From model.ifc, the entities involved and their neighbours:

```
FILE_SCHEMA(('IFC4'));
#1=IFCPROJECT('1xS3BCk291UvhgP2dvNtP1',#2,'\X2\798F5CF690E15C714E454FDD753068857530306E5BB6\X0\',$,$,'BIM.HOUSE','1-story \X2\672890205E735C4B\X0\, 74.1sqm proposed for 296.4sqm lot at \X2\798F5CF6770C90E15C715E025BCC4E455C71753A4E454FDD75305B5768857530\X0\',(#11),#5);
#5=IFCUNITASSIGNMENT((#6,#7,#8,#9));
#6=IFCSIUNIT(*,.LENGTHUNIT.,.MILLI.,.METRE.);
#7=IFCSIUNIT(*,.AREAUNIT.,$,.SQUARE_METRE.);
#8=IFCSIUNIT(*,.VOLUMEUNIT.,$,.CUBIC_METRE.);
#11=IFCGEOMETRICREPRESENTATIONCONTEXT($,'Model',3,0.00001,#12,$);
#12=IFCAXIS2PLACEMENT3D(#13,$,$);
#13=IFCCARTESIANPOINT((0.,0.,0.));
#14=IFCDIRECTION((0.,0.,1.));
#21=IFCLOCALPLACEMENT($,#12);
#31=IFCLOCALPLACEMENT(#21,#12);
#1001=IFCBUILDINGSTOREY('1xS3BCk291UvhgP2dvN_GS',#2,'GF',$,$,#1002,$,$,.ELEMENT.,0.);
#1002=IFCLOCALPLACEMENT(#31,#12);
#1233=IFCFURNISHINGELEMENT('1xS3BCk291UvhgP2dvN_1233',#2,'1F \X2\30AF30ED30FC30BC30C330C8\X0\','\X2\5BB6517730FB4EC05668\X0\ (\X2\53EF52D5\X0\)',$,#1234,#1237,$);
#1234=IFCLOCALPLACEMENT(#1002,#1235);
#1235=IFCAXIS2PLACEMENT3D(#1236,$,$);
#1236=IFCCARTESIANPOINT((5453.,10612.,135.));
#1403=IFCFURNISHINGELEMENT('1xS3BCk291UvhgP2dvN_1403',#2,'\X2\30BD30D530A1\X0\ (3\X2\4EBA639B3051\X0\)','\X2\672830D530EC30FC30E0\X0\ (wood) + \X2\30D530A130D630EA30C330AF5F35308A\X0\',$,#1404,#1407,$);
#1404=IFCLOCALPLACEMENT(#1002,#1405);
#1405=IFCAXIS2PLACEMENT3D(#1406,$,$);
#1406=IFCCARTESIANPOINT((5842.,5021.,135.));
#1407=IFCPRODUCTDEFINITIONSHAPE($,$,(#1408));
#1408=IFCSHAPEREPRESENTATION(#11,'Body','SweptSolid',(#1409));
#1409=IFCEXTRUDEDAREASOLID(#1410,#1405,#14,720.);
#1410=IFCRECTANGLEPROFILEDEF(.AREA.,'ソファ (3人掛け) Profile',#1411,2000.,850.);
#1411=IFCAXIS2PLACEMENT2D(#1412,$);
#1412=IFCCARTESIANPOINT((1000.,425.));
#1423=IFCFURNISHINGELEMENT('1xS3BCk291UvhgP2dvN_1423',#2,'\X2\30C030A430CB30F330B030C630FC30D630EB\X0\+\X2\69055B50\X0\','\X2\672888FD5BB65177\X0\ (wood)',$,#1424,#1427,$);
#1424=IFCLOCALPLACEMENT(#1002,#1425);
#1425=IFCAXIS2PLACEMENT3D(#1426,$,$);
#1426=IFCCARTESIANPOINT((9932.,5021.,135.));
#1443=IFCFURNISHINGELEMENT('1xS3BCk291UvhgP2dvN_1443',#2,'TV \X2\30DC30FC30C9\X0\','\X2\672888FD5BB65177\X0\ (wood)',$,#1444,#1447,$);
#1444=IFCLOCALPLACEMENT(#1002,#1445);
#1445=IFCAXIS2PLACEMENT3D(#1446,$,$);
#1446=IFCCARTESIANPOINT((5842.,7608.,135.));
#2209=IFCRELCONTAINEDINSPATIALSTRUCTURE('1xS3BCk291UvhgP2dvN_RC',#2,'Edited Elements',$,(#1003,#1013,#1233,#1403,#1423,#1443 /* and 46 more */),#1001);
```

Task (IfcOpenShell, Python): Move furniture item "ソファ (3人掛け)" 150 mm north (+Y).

```python
import ifcopenshell
import ifcopenshell.api.geometry
import ifcopenshell.util.placement

model = ifcopenshell.open("model.ifc")

item = model.by_guid("1xS3BCk291UvhgP2dvN_1403")
matrix = ifcopenshell.util.placement.get_local_placement(item.ObjectPlacement)
matrix[1, 3] += 150.0
ifcopenshell.api.geometry.edit_object_placement(model, product=item, matrix=matrix, is_si=False)

print(ifcopenshell.util.placement.get_local_placement(item.ObjectPlacement).round(3) + 0.0)

model.write("model_updated.ifc")
```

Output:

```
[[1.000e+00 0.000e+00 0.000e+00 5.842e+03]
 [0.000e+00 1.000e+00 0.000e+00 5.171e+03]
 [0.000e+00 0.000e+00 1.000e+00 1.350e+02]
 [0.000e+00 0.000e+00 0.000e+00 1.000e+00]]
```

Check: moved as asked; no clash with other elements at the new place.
